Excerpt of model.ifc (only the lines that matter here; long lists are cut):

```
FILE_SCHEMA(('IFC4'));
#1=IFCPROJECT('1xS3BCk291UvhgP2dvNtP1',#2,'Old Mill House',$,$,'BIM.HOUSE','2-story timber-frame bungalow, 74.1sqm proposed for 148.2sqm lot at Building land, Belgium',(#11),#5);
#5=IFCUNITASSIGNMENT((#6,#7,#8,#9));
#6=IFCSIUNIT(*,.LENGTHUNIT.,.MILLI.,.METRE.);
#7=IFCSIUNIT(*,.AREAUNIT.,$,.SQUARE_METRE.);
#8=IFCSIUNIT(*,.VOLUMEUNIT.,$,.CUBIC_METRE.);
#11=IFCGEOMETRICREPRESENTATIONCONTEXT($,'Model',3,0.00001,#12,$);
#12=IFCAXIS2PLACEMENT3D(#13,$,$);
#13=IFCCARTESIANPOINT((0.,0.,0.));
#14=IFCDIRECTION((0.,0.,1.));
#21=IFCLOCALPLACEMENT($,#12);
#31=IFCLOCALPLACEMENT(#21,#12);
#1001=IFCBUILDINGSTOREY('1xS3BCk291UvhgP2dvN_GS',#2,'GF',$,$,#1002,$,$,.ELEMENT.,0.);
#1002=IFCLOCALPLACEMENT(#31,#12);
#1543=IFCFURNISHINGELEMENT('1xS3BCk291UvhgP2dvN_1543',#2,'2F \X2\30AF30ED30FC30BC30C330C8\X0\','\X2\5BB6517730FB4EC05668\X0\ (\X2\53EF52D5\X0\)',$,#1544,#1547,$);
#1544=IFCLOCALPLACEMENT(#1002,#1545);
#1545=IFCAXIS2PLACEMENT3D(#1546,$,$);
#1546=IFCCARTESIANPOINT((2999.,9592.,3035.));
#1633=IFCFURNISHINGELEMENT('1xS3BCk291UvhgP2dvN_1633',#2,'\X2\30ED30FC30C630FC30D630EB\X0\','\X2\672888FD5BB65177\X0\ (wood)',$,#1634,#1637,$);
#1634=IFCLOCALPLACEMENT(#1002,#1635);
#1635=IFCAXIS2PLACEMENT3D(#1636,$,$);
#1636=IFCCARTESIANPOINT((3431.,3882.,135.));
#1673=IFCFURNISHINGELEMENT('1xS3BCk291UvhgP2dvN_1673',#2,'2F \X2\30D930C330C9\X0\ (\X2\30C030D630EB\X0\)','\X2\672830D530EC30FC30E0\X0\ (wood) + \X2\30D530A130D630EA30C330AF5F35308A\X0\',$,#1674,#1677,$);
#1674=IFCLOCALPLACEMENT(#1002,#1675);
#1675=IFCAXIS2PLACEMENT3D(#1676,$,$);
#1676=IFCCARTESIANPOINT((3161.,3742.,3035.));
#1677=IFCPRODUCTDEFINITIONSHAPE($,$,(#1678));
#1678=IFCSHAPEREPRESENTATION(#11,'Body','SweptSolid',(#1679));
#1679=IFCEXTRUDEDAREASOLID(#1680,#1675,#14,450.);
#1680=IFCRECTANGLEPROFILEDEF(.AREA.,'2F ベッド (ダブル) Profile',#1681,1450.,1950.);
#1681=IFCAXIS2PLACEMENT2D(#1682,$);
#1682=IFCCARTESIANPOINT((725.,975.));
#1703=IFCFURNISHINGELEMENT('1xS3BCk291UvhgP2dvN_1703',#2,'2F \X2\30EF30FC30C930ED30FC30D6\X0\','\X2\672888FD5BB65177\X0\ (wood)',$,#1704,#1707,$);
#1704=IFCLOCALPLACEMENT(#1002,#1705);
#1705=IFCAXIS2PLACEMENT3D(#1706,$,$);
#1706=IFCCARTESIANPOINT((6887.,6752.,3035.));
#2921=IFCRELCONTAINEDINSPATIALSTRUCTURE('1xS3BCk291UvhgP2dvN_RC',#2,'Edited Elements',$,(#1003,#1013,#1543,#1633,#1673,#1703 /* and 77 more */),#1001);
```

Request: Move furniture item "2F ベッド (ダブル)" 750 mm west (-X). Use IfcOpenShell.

```python
import ifcopenshell
import ifcopenshell.api.geometry
import ifcopenshell.util.placement

model = ifcopenshell.open("model.ifc")

item = model.by_guid("1xS3BCk291UvhgP2dvN_1673")
matrix = ifcopenshell.util.placement.get_local_placement(item.ObjectPlacement)
matrix[0, 3] -= 750.0
ifcopenshell.api.geometry.edit_object_placement(model, product=item, matrix=matrix, is_si=False)

print(ifcopenshell.util.placement.get_local_placement(item.ObjectPlacement).round(3) + 0.0)

model.write("model-out.ifc")
```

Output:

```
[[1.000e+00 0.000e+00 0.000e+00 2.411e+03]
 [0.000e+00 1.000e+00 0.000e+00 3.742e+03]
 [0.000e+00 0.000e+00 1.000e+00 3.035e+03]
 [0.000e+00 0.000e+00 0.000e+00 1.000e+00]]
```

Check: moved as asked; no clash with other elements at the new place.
